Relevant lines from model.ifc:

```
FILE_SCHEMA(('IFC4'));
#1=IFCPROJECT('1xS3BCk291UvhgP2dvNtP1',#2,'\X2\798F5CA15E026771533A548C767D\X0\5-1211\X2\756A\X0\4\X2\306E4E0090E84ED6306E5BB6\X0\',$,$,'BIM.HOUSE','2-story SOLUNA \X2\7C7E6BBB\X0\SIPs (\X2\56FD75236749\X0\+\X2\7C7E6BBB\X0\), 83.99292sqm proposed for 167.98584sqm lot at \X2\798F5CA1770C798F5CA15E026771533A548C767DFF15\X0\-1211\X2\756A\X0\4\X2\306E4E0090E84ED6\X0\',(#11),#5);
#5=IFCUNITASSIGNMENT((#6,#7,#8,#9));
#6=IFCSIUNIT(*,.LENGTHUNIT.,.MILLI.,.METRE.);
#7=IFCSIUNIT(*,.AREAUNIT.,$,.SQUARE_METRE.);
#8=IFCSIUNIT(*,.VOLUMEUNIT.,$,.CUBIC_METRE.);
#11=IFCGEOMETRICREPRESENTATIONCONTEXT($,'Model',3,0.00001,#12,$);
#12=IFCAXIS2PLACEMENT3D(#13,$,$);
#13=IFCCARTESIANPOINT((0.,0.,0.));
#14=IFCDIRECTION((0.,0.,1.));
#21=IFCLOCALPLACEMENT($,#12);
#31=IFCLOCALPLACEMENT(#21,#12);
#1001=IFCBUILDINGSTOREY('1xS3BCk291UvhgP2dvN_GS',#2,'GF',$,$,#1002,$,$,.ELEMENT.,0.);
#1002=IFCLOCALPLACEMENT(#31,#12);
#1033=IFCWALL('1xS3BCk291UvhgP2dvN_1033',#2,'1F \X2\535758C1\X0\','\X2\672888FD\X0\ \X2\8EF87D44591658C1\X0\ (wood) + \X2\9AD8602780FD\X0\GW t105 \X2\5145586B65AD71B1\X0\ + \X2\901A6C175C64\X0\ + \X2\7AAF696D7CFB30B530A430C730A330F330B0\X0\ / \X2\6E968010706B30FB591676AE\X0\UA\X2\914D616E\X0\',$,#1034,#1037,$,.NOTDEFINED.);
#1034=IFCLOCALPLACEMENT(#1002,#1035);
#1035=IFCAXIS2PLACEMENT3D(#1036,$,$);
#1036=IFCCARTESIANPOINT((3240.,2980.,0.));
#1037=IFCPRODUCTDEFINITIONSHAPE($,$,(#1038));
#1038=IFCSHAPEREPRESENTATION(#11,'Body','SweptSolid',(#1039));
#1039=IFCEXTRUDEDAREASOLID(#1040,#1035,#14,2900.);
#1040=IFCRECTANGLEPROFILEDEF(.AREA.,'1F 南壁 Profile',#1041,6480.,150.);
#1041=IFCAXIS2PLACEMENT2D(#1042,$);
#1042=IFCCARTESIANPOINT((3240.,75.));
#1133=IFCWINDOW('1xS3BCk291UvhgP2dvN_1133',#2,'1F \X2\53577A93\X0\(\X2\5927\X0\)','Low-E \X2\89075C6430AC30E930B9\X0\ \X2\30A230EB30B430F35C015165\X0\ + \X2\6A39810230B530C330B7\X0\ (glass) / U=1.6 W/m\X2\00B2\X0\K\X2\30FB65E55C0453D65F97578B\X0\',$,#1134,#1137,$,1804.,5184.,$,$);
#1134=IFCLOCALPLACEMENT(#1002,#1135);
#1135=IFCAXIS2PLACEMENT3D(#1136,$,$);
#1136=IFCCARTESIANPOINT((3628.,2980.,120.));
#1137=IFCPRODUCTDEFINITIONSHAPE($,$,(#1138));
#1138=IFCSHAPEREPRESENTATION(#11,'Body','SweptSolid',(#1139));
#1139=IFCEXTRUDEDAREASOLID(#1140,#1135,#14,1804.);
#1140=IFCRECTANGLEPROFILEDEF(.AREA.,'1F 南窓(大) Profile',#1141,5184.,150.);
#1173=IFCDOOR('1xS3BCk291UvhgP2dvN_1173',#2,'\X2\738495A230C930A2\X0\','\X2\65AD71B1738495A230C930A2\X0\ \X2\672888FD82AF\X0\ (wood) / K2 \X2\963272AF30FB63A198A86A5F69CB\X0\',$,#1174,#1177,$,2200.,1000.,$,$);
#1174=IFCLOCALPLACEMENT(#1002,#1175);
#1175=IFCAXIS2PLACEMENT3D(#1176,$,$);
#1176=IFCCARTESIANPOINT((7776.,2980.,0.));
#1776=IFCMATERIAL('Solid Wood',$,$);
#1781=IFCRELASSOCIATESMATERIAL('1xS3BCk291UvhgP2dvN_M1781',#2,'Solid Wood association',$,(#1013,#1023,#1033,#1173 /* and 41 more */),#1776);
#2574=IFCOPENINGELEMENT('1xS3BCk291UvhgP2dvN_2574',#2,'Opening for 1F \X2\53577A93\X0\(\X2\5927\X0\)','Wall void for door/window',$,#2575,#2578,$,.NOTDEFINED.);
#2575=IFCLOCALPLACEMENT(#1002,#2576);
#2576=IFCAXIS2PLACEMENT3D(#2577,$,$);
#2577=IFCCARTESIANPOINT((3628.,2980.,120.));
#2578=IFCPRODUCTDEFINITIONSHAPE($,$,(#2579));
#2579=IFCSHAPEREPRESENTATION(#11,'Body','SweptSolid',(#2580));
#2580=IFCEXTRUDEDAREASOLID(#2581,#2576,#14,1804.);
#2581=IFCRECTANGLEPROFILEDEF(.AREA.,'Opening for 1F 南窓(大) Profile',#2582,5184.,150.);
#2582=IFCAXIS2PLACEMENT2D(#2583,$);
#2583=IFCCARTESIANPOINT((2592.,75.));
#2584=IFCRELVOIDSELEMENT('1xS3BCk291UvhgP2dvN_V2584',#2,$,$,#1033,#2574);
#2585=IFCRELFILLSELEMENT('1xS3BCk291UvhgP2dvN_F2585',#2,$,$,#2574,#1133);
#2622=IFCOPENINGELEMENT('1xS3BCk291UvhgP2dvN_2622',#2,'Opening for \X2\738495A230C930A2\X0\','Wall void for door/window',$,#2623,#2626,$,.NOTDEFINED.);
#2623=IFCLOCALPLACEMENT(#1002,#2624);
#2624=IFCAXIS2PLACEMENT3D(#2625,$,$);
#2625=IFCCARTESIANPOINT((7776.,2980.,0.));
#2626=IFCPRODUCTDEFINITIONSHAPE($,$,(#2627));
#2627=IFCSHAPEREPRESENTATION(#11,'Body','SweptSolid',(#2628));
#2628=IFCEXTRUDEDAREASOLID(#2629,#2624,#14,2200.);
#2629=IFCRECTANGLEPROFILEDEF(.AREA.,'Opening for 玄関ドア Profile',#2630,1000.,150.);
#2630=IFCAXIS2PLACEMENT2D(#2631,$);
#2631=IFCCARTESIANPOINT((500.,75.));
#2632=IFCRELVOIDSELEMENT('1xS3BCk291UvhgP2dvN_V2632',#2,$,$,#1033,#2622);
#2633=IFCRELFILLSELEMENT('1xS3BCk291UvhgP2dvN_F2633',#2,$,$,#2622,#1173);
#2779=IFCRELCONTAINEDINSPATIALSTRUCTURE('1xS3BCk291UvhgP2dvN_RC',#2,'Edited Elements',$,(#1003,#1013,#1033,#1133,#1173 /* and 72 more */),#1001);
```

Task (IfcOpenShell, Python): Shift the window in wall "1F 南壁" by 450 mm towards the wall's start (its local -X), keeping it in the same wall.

```python
import ifcopenshell
import ifcopenshell.api.geometry
import ifcopenshell.util.placement
import ifcopenshell.util.unit

model = ifcopenshell.open("model.ifc")
unit_scale = ifcopenshell.util.unit.calculate_unit_scale(model)

window = model.by_guid("1xS3BCk291UvhgP2dvN_1133")
opening = window.FillsVoids[0].RelatingOpeningElement
wall = opening.VoidsElements[0].RelatingBuildingElement

wall_matrix = ifcopenshell.util.placement.get_local_placement(wall.ObjectPlacement)
shift = wall_matrix[:3, 0] * -0.45 / unit_scale
before = ifcopenshell.util.placement.get_local_placement(window.ObjectPlacement)[:3, 3].copy()

# The window is not placed relative to its opening, so move both.
for product in (opening, window):
    matrix = ifcopenshell.util.placement.get_local_placement(product.ObjectPlacement)
    matrix[:3, 3] += shift
    ifcopenshell.api.geometry.edit_object_placement(model, product=product, matrix=matrix, is_si=False)

after = ifcopenshell.util.placement.get_local_placement(window.ObjectPlacement)[:3, 3]
print("window moved by", (after - before).round(3) + 0.0)

model.write("model_rev.ifc")
```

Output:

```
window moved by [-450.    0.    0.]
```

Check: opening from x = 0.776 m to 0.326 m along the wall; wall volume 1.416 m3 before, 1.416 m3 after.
